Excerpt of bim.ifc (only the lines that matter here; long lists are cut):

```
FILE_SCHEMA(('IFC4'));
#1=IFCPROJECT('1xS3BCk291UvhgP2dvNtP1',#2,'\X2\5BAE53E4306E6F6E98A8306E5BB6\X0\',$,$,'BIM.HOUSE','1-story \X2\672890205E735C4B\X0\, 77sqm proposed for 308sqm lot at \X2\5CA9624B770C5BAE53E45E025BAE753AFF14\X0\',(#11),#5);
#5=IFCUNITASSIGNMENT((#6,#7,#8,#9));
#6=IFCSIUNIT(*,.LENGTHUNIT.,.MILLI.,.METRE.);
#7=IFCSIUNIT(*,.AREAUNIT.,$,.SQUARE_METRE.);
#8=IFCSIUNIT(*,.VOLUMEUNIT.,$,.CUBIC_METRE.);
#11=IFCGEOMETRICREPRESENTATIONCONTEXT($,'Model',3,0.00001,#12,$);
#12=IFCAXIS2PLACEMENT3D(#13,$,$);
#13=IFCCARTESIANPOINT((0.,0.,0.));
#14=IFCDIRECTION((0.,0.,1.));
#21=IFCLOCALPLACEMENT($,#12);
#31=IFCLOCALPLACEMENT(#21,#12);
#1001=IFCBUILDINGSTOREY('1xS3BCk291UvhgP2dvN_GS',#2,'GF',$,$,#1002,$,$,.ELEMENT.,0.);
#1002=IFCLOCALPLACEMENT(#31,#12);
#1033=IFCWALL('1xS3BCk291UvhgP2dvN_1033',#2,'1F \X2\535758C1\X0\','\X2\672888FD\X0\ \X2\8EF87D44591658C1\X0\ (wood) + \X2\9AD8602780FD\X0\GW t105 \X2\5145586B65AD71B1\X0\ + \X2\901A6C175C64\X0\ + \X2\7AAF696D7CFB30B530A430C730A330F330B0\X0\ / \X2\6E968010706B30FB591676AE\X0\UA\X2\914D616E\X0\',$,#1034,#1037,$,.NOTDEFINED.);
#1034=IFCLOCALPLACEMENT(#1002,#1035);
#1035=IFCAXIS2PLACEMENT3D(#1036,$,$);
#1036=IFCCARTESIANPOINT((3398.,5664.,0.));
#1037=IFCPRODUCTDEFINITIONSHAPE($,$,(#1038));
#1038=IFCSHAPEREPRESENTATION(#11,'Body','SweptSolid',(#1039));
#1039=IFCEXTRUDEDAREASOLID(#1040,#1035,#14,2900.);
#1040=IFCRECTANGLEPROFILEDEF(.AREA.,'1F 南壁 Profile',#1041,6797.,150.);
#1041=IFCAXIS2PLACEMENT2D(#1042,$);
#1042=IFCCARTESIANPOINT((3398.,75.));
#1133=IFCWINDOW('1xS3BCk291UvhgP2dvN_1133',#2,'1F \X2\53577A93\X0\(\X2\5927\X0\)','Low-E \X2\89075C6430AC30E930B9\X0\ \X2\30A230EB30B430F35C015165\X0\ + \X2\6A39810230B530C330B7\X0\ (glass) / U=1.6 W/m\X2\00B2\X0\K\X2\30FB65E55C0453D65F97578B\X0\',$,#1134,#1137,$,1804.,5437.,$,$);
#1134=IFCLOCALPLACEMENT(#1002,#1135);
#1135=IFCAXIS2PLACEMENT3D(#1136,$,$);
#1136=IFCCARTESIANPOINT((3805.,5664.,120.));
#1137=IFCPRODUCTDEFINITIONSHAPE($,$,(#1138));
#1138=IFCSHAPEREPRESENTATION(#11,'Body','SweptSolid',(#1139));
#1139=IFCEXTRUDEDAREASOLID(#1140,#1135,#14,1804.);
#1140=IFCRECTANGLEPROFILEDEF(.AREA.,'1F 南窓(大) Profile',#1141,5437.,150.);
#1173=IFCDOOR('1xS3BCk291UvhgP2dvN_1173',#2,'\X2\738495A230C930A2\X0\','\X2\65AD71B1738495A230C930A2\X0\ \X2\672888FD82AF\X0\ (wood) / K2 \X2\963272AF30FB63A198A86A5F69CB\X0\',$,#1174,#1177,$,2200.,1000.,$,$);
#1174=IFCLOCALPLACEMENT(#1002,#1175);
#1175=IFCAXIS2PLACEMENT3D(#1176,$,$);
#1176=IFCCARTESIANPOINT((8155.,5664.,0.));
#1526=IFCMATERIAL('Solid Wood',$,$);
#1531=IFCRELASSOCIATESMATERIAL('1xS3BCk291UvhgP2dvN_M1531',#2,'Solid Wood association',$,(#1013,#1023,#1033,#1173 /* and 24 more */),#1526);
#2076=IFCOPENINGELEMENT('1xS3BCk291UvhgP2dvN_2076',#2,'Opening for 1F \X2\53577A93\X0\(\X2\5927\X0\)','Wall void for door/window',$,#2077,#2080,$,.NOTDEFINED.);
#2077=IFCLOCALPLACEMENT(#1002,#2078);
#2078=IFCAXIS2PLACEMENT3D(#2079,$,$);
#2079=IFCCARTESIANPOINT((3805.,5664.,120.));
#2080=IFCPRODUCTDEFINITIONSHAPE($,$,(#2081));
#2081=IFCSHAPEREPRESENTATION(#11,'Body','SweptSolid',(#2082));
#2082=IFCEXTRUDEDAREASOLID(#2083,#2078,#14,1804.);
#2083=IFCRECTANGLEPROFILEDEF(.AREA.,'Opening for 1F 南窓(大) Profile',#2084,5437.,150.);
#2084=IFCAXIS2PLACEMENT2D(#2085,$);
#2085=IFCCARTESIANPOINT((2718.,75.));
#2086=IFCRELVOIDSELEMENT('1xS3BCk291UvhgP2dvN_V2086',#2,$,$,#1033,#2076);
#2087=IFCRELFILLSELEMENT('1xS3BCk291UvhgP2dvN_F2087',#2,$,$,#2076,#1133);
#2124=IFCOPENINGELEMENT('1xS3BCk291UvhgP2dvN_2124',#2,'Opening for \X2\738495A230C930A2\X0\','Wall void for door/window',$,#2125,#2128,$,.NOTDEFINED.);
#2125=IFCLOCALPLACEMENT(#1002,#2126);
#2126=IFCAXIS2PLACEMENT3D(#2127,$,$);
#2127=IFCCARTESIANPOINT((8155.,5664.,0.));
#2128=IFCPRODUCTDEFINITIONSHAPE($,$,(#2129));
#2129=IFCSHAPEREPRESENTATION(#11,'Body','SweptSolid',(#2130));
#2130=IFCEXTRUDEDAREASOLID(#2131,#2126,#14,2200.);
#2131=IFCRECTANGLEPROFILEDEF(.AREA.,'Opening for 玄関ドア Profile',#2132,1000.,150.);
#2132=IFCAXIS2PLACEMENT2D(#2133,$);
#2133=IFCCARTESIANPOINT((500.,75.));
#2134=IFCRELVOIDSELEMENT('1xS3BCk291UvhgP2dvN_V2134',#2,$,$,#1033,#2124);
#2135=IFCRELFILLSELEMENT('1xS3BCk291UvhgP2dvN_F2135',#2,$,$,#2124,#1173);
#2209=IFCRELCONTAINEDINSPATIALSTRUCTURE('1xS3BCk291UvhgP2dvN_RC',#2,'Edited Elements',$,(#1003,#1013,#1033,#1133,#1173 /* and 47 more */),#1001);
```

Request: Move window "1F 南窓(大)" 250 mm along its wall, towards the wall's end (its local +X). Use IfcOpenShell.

```python
import ifcopenshell
import ifcopenshell.api.geometry
import ifcopenshell.util.placement

model = ifcopenshell.open("bim.ifc")

window = model.by_id(1133)
opening = window.FillsVoids[0].RelatingOpeningElement
wall = opening.VoidsElements[0].RelatingBuildingElement

wall_matrix = ifcopenshell.util.placement.get_local_placement(wall.ObjectPlacement)
shift = wall_matrix[:3, 0] * 250.0
before = ifcopenshell.util.placement.get_local_placement(window.ObjectPlacement)[:3, 3].copy()

# The window is not placed relative to its opening, so move both.
for product in (opening, window):
    matrix = ifcopenshell.util.placement.get_local_placement(product.ObjectPlacement)
    matrix[:3, 3] += shift
    ifcopenshell.api.geometry.edit_object_placement(model, product=product, matrix=matrix, is_si=False)

after = ifcopenshell.util.placement.get_local_placement(window.ObjectPlacement)[:3, 3]
print("window moved by", (after - before).round(3) + 0.0)

model.write("bim_v2.ifc")
```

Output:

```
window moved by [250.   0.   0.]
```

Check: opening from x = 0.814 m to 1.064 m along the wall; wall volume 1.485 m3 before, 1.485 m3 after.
